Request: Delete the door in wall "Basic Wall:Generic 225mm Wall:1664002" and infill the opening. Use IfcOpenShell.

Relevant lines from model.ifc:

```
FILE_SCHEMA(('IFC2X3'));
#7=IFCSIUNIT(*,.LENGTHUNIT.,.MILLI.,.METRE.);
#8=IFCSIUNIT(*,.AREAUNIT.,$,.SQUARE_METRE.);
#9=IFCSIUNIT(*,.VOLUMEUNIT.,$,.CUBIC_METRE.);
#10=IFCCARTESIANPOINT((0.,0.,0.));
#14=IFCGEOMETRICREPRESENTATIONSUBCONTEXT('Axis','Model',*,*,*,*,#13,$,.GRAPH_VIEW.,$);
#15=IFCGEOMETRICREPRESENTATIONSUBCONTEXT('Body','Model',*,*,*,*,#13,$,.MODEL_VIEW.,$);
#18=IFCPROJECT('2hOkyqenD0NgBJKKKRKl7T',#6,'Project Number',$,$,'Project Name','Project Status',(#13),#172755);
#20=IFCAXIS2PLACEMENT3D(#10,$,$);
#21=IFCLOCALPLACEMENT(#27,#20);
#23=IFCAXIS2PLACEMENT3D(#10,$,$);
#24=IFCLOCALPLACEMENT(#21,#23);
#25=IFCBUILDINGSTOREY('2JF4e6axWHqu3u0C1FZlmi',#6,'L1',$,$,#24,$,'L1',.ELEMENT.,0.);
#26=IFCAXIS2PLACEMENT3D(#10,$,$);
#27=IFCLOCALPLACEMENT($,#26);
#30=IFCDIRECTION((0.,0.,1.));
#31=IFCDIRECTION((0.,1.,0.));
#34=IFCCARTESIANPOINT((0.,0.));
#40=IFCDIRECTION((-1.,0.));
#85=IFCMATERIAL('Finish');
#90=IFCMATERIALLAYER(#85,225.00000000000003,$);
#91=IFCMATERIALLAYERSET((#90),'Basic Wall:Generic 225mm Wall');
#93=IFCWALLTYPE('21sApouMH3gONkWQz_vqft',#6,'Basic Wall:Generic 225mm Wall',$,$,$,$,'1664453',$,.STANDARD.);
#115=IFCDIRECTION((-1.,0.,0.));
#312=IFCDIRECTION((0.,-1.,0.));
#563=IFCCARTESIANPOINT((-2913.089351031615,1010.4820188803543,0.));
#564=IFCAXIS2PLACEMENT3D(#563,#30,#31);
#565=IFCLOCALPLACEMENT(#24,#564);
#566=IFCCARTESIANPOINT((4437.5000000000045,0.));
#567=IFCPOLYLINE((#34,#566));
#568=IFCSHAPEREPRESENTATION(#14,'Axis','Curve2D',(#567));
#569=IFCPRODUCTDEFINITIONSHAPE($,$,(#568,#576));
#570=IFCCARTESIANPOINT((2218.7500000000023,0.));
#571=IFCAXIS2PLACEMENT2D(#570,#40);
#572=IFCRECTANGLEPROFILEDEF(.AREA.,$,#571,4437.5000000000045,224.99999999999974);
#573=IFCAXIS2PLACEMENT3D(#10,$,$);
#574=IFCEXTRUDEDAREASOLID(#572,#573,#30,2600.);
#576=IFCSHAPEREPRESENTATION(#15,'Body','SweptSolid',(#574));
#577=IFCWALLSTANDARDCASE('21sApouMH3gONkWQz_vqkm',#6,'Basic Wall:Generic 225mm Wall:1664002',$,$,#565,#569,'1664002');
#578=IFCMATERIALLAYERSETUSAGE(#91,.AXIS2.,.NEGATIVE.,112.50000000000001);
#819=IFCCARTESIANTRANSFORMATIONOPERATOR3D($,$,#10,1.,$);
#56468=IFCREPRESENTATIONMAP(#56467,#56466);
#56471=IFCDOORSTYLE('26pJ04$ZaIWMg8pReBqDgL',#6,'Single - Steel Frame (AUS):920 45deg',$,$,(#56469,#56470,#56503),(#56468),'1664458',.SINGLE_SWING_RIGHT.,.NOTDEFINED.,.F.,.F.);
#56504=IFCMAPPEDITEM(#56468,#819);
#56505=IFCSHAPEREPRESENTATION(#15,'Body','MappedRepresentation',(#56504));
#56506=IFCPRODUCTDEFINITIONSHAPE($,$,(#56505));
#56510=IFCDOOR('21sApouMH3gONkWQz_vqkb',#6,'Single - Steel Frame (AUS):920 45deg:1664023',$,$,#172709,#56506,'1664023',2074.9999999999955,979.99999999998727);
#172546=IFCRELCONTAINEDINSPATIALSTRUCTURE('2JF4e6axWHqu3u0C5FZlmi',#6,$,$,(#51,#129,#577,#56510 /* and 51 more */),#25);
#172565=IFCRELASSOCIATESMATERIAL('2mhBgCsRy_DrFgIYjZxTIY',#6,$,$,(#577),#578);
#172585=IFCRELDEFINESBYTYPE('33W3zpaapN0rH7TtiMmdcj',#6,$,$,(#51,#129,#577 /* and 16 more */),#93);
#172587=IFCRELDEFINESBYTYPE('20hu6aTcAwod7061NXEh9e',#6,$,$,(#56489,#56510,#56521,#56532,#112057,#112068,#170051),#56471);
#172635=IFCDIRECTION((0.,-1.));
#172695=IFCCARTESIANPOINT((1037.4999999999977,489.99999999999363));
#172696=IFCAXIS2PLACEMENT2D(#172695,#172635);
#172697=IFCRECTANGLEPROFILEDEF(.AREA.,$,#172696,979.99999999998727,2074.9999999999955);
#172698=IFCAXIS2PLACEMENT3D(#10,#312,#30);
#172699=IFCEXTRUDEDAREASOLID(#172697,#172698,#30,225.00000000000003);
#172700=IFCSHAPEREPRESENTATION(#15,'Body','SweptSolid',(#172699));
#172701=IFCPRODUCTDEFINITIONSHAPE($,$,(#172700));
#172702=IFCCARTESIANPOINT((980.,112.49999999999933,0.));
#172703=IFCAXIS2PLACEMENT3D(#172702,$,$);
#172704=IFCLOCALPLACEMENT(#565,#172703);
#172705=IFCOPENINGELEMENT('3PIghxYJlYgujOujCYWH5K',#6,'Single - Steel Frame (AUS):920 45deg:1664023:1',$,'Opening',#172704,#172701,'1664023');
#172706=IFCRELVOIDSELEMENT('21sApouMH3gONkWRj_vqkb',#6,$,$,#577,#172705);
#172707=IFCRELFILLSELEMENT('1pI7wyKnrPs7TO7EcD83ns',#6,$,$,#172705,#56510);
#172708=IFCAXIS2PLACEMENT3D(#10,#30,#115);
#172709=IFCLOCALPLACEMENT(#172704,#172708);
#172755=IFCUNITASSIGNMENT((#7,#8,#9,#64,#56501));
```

```python
import ifcopenshell
import ifcopenshell.api.feature
import ifcopenshell.api.root
import ifcopenshell.geom
import ifcopenshell.util.shape

model = ifcopenshell.open("model.ifc")
settings = ifcopenshell.geom.settings()


def volume(element):
    """Net volume in cubic metres, openings subtracted."""
    shape = ifcopenshell.geom.create_shape(settings, element)
    return ifcopenshell.util.shape.get_volume(shape.geometry)


door = model.by_guid("21sApouMH3gONkWQz_vqkb")
opening = door.FillsVoids[0].RelatingOpeningElement
wall = opening.VoidsElements[0].RelatingBuildingElement
before = volume(wall)

ifcopenshell.api.root.remove_product(model, product=door)
ifcopenshell.api.feature.remove_feature(model, feature=opening)

after = volume(wall)

print(f"wall volume {before:.3f} -> {after:.3f} m3")

model.write("model-out.ifc")
```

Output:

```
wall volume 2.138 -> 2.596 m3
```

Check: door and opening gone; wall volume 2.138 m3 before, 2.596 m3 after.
